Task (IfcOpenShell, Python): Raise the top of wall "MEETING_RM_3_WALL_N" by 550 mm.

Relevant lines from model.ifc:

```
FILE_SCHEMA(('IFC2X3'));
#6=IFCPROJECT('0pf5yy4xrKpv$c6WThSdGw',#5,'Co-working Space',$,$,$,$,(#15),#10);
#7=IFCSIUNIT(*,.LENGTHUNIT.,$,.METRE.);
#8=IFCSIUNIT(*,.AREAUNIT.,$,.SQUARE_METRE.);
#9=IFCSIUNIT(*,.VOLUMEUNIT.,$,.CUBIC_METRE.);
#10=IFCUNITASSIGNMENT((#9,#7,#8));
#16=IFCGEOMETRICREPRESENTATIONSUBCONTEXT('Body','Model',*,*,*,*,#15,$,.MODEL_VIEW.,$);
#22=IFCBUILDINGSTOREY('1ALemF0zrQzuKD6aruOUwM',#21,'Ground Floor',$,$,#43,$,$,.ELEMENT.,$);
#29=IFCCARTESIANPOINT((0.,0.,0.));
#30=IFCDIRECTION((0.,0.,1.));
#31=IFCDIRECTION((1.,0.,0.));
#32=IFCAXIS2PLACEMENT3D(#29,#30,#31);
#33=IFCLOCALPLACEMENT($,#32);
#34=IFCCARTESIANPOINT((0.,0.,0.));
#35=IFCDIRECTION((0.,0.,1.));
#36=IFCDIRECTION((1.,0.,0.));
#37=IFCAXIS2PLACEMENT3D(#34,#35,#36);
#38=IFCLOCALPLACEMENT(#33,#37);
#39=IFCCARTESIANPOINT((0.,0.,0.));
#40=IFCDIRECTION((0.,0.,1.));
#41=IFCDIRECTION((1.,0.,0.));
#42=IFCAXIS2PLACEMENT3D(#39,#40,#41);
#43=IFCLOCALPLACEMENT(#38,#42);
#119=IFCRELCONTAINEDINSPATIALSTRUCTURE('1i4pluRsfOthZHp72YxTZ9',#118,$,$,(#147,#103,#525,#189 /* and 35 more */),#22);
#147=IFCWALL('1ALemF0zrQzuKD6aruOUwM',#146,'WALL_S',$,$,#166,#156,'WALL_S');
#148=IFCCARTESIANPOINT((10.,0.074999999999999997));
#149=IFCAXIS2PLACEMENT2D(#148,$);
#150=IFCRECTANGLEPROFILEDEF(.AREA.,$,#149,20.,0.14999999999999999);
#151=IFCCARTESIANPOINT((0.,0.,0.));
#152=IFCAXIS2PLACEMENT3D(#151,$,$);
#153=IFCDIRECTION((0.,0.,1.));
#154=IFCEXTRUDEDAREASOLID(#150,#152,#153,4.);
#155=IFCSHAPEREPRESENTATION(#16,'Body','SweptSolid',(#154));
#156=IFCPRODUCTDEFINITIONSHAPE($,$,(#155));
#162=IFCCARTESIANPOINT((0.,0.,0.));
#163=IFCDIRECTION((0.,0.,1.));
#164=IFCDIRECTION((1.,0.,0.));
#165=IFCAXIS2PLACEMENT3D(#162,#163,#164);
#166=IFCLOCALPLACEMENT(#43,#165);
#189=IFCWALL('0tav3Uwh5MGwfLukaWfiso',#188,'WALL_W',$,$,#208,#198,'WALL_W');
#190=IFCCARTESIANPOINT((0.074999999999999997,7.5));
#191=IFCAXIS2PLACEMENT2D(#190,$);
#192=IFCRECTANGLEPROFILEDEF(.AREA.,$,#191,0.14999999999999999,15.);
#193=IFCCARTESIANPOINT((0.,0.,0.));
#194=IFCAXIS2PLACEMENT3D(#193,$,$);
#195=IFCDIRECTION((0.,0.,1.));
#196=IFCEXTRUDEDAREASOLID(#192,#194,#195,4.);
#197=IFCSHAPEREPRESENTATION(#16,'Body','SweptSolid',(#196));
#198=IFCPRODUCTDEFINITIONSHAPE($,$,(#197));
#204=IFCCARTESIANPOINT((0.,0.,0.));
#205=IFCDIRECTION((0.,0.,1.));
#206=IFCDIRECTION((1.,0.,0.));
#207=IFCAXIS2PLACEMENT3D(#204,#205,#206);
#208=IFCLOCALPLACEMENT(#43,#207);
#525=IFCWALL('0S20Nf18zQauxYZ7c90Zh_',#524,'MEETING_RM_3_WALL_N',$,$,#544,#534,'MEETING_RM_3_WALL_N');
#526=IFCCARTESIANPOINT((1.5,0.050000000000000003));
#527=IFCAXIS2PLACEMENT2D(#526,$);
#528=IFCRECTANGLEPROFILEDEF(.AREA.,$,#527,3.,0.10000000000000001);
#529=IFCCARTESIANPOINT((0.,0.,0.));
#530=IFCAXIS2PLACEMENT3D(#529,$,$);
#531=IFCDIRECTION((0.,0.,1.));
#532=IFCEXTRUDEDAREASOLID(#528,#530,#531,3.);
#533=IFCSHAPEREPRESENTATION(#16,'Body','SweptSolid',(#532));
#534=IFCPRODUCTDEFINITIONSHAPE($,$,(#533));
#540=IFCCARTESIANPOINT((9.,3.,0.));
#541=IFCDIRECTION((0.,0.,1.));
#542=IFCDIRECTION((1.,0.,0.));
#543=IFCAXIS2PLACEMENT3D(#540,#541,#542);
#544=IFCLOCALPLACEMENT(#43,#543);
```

```python
import ifcopenshell
import ifcopenshell.geom
import ifcopenshell.util.representation
import ifcopenshell.util.shape
import ifcopenshell.util.unit

model = ifcopenshell.open("model.ifc")
unit_scale = ifcopenshell.util.unit.calculate_unit_scale(model)
settings = ifcopenshell.geom.settings()


def volume(element):
    """Net volume in cubic metres, openings subtracted."""
    shape = ifcopenshell.geom.create_shape(settings, element)
    return ifcopenshell.util.shape.get_volume(shape.geometry)


wall = model.by_id(525)
before = volume(wall)

body = ifcopenshell.util.representation.get_representation(wall, "Model", "Body")
solid = body.Items[0]
old_height = solid.Depth
solid.Depth += 0.55 / unit_scale
after = volume(wall)

print(f"height {old_height:g} -> {solid.Depth:g}, volume {before:.3f} -> {after:.3f} m3")

model.write("model_v2.ifc")
```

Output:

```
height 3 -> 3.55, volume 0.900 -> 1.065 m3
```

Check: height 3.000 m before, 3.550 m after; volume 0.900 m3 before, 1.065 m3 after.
